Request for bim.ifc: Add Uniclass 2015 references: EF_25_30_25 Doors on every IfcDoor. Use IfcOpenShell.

First a look at what the model holds.

```python
import ifcopenshell

model = ifcopenshell.open("bim.ifc")
print(model.schema)
print("classifications:", [c.Name for c in model.by_type("IfcClassification")])
for ifc_class in ("IfcDoor", "IfcRoof", "IfcStair", "IfcWall", "IfcWindow"):
    print(ifc_class, len(model.by_type(ifc_class)))
```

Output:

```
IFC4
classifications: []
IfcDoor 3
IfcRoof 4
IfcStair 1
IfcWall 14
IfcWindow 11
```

```python
import ifcopenshell
import ifcopenshell.api.classification

model = ifcopenshell.open("bim.ifc")

system = ifcopenshell.api.classification.add_classification(model, classification="Uniclass 2015")

codes = {
    "IfcDoor": ("EF_25_30_25", "Doors"),
}
for ifc_class, (code, name) in codes.items():
    products = model.by_type(ifc_class)
    ifcopenshell.api.classification.add_reference(
        model, products=products, classification=system, identification=code, name=name
    )
    print(code, len(products))

model.write("bim_v2.ifc")
```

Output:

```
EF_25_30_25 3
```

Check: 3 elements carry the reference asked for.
